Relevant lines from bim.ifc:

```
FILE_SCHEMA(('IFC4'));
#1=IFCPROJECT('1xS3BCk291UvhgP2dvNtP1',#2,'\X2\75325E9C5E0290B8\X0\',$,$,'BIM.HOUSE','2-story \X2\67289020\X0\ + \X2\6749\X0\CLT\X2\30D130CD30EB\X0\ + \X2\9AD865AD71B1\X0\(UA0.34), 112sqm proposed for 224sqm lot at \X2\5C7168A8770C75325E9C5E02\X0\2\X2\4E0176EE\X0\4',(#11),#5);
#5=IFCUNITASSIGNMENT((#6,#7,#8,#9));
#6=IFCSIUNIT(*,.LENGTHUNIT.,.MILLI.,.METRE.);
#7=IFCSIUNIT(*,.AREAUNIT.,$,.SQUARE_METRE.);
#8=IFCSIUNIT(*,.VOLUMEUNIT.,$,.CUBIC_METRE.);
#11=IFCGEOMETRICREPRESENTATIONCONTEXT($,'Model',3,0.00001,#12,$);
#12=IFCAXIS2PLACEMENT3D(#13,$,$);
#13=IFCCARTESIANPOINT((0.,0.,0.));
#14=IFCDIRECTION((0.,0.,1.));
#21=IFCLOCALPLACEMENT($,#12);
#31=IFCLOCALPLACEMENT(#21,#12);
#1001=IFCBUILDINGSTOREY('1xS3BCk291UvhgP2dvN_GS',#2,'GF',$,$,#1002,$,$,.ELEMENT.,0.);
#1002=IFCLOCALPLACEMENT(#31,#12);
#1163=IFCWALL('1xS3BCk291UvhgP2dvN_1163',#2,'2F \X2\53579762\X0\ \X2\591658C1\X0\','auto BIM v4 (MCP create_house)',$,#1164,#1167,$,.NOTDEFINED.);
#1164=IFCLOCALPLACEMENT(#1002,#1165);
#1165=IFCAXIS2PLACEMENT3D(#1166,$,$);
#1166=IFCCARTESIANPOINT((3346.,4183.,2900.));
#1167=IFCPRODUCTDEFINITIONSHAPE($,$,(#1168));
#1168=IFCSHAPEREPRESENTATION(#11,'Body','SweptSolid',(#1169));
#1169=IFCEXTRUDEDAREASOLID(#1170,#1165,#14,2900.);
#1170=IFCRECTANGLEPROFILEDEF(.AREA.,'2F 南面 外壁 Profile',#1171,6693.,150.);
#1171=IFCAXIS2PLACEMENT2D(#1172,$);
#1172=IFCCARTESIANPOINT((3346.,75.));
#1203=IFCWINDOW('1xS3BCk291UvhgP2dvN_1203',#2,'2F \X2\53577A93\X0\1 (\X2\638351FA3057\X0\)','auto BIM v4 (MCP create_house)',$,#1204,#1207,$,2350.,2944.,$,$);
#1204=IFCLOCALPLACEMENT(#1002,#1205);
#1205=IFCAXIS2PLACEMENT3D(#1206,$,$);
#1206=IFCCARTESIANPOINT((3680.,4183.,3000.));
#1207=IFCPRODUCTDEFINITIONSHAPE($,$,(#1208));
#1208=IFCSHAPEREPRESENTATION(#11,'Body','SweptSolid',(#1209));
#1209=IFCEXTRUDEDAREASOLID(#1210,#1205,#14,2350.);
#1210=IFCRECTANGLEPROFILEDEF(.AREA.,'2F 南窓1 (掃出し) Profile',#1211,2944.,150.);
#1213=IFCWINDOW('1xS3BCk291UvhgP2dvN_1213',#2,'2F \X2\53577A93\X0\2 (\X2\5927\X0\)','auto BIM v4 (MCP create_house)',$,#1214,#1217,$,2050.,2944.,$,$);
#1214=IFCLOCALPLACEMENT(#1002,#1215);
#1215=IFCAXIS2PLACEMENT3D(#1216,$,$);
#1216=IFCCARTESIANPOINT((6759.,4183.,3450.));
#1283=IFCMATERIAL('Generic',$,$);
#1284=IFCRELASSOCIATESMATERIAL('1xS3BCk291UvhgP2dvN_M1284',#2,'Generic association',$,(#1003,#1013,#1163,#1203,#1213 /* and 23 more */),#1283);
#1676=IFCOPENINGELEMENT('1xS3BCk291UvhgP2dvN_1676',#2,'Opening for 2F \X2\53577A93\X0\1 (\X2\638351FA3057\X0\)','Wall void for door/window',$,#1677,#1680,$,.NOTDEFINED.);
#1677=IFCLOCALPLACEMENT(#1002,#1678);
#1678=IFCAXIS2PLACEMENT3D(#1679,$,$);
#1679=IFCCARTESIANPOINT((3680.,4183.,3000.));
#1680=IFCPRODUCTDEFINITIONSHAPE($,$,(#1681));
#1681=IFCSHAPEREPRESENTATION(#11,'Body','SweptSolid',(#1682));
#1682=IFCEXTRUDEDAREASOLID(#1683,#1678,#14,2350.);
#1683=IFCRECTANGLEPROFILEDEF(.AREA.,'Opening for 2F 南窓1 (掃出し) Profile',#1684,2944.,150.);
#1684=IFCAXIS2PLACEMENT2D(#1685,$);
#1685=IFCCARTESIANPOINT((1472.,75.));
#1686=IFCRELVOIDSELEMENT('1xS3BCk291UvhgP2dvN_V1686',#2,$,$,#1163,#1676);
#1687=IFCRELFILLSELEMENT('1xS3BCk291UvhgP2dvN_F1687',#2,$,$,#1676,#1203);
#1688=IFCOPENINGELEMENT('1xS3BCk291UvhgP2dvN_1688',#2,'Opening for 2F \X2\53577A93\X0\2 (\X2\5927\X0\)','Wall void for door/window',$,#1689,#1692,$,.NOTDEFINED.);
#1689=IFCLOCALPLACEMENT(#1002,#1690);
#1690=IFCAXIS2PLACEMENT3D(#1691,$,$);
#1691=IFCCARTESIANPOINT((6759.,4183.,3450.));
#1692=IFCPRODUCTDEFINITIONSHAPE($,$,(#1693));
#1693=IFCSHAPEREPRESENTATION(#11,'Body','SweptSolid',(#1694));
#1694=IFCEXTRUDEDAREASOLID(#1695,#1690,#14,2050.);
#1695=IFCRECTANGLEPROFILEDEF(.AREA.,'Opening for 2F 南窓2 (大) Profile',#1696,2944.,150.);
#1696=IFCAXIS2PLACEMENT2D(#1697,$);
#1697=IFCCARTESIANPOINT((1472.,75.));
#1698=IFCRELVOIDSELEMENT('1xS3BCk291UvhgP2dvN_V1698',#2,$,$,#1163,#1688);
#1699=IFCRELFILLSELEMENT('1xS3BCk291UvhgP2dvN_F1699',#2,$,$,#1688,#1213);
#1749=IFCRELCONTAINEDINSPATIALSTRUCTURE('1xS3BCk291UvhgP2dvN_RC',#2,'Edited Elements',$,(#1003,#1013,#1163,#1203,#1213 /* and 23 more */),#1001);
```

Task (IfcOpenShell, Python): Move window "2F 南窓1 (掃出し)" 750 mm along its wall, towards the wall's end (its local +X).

```python
import ifcopenshell
import ifcopenshell.api.geometry
import ifcopenshell.util.placement

model = ifcopenshell.open("bim.ifc")

window = model.by_guid("1xS3BCk291UvhgP2dvN_1203")
opening = window.FillsVoids[0].RelatingOpeningElement
wall = opening.VoidsElements[0].RelatingBuildingElement

wall_matrix = ifcopenshell.util.placement.get_local_placement(wall.ObjectPlacement)
shift = wall_matrix[:3, 0] * 750.0
before = ifcopenshell.util.placement.get_local_placement(window.ObjectPlacement)[:3, 3].copy()

# The window is not placed relative to its opening, so move both.
for product in (opening, window):
    matrix = ifcopenshell.util.placement.get_local_placement(product.ObjectPlacement)
    matrix[:3, 3] += shift
    ifcopenshell.api.geometry.edit_object_placement(model, product=product, matrix=matrix, is_si=False)

after = ifcopenshell.util.placement.get_local_placement(window.ObjectPlacement)[:3, 3]
print("window moved by", (after - before).round(3) + 0.0)

model.write("bim_updated.ifc")
```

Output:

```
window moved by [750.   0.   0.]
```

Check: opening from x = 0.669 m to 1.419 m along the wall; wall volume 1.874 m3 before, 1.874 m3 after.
